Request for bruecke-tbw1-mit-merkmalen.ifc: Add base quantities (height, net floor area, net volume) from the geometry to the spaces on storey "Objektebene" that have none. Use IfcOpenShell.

First a look at what the model holds.

```python
import ifcopenshell
import ifcopenshell.util.element
import ifcopenshell.util.unit

model = ifcopenshell.open("bruecke-tbw1-mit-merkmalen.ifc")
print(model.schema)
for unit_type in ("LENGTHUNIT", "AREAUNIT", "VOLUMEUNIT"):
    print(unit_type, ifcopenshell.util.unit.calculate_unit_scale(model, unit_type))
storey = next(s for s in model.by_type("IfcBuildingStorey") if s.Name == "Objektebene")
spaces = [e for e in ifcopenshell.util.element.get_decomposition(storey) if e.is_a("IfcSpace")]
for e in sorted(spaces, key=lambda e: e.id()):
    print(e.id(), e.is_a(), e.Name, list(ifcopenshell.util.element.get_psets(e, qtos_only=True)), sep=" | ")
```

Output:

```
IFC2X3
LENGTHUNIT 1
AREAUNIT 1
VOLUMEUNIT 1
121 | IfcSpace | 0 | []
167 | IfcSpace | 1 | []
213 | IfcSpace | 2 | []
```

```python
import ifcopenshell
import ifcopenshell.api.pset
import ifcopenshell.geom
import ifcopenshell.util.element
import ifcopenshell.util.shape
import ifcopenshell.util.unit

model = ifcopenshell.open("bruecke-tbw1-mit-merkmalen.ifc")
unit_scale = ifcopenshell.util.unit.calculate_unit_scale(model)
area_scale = ifcopenshell.util.unit.calculate_unit_scale(model, "AREAUNIT")
volume_scale = ifcopenshell.util.unit.calculate_unit_scale(model, "VOLUMEUNIT")
settings = ifcopenshell.geom.settings()

storey = next(s for s in model.by_type("IfcBuildingStorey") if s.Name == "Objektebene")
spaces = [e for e in ifcopenshell.util.element.get_decomposition(storey) if e.is_a("IfcSpace")]

for e in sorted(spaces, key=lambda e: e.id()):
    if ifcopenshell.util.element.get_psets(e, qtos_only=True, should_inherit=False):
        continue
    # Geometry comes back in metres, in the element's own axes.
    shape = ifcopenshell.geom.create_shape(settings, e)
    values = {
        "Height": ifcopenshell.util.shape.get_z(shape.geometry) / unit_scale,
        "NetFloorArea": ifcopenshell.util.shape.get_footprint_area(shape.geometry) / area_scale,
        "NetVolume": ifcopenshell.util.shape.get_volume(shape.geometry) / volume_scale,
    }
    qto = ifcopenshell.api.pset.add_qto(model, product=e, name="BaseQuantities")
    ifcopenshell.api.pset.edit_qto(model, qto=qto, properties=values)
    print(e.id(), {k: round(v, 3) for k, v in values.items()})

model.write("bruecke-tbw1-mit-merkmalen_rev.ifc")
```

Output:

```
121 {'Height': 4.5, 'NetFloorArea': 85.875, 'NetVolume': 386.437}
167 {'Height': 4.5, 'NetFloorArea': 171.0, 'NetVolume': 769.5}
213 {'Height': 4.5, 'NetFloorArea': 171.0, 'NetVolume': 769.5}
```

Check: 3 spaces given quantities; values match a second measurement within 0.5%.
